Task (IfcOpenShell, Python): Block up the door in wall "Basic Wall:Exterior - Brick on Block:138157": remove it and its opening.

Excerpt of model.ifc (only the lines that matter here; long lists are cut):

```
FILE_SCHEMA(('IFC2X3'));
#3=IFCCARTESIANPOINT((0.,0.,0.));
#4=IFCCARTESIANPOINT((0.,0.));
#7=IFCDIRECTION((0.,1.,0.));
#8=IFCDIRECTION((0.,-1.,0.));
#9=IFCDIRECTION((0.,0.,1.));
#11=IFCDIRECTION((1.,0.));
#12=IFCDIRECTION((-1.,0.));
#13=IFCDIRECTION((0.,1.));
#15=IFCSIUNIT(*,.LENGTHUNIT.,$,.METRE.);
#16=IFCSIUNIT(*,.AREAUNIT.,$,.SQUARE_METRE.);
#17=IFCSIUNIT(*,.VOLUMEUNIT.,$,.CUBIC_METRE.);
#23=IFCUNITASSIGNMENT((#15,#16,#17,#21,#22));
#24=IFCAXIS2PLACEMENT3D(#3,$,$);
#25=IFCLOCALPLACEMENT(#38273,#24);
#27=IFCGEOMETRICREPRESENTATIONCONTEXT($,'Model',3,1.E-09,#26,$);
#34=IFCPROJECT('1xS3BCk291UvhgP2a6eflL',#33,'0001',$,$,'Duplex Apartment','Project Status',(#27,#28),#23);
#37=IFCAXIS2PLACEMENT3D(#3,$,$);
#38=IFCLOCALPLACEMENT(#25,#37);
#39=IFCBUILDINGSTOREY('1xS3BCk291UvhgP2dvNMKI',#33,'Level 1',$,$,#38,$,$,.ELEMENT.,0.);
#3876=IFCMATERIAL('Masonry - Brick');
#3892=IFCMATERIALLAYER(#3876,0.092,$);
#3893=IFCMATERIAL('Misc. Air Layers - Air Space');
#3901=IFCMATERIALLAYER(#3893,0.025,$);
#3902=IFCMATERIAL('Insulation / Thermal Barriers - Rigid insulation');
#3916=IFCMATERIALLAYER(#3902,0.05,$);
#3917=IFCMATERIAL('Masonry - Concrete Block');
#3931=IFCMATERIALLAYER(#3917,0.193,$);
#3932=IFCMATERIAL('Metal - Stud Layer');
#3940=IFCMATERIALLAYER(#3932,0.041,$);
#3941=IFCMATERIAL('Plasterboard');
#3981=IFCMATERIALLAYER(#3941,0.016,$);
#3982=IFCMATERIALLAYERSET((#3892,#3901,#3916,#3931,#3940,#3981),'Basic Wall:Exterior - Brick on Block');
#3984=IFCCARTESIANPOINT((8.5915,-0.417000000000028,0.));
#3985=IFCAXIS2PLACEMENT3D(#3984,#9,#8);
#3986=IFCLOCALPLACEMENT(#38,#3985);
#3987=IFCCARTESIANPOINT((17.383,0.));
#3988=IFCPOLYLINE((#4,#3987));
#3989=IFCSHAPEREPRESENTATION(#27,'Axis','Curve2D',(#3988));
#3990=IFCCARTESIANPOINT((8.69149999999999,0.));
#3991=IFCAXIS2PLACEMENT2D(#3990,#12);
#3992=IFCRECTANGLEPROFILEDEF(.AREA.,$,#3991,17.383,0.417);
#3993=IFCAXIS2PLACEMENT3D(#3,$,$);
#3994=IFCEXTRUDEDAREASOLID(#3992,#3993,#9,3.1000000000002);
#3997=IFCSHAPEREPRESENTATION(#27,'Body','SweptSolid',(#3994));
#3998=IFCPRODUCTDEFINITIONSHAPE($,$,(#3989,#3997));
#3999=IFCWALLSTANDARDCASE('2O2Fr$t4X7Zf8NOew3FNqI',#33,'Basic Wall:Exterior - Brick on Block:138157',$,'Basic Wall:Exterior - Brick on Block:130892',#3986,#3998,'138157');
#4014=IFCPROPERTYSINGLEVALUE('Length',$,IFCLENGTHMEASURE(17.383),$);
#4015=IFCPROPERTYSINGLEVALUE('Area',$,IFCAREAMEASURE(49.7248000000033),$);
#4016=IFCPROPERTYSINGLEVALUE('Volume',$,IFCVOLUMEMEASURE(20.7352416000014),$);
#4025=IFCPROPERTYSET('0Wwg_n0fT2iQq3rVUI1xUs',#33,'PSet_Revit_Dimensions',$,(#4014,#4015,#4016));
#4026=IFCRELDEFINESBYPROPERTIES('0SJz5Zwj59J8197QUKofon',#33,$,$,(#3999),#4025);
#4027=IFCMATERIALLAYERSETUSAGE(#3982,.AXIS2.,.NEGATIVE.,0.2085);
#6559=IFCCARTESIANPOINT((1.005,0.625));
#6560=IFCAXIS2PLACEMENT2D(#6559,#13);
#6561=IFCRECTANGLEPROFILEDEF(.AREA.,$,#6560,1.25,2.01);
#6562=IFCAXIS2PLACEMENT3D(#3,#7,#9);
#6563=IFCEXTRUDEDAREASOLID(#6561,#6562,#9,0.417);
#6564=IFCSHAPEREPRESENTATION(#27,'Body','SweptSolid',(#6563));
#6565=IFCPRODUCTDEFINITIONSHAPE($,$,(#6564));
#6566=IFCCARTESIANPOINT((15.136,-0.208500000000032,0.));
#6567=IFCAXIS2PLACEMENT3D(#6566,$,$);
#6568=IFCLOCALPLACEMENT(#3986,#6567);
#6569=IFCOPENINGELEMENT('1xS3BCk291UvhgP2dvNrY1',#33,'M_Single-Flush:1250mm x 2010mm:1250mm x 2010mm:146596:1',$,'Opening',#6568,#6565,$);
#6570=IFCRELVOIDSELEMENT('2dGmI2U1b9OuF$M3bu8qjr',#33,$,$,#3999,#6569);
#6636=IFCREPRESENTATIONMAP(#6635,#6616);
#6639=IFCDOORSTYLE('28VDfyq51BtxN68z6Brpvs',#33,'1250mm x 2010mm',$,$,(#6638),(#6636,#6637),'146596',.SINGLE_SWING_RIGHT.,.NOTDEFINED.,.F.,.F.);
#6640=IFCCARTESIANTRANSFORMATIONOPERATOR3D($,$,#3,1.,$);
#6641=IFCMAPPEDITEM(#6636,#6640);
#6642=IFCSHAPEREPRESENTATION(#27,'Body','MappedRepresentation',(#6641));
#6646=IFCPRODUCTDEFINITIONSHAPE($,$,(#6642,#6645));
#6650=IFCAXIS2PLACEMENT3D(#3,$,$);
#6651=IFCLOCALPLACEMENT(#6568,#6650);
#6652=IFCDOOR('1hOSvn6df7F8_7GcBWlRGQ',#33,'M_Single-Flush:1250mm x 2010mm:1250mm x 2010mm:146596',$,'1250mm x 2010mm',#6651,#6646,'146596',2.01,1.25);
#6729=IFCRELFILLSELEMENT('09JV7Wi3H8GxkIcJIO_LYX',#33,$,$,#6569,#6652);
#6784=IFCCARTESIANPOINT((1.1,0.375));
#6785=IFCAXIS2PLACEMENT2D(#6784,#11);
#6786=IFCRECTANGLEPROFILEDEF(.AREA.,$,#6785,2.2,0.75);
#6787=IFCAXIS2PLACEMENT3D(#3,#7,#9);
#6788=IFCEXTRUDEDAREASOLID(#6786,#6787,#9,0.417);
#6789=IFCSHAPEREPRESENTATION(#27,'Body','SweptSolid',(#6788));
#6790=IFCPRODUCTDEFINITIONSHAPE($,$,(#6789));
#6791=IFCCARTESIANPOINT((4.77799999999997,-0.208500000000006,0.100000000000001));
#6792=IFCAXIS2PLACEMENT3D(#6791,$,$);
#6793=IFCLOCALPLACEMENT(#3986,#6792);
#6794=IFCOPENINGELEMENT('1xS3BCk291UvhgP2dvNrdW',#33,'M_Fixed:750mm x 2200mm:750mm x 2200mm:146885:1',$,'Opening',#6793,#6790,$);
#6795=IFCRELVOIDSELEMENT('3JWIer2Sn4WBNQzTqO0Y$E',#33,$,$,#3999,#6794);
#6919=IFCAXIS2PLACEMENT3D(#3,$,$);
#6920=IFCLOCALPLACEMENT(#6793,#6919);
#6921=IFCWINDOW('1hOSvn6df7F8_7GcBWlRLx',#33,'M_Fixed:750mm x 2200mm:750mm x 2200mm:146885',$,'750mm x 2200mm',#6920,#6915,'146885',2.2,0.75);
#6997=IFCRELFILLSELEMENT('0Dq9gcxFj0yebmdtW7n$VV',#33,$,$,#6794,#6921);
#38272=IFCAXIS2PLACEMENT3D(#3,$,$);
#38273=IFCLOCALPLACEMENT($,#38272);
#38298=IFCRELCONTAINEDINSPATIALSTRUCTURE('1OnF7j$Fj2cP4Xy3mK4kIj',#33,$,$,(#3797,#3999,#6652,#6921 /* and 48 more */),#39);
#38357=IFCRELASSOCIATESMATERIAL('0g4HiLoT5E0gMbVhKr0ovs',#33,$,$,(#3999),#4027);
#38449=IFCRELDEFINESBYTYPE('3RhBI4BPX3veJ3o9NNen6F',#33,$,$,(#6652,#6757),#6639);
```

```python
import ifcopenshell
import ifcopenshell.api.feature
import ifcopenshell.api.pset
import ifcopenshell.api.root
import ifcopenshell.geom
import ifcopenshell.util.element
import ifcopenshell.util.shape
import ifcopenshell.util.unit

model = ifcopenshell.open("model.ifc")
area_scale = ifcopenshell.util.unit.calculate_unit_scale(model, "AREAUNIT")
volume_scale = ifcopenshell.util.unit.calculate_unit_scale(model, "VOLUMEUNIT")
settings = ifcopenshell.geom.settings()


def volume(element):
    """Net volume in cubic metres, openings subtracted."""
    shape = ifcopenshell.geom.create_shape(settings, element)
    return ifcopenshell.util.shape.get_volume(shape.geometry)


door = model.by_id(6652)
opening = door.FillsVoids[0].RelatingOpeningElement
wall = opening.VoidsElements[0].RelatingBuildingElement
before = volume(wall)

ifcopenshell.api.root.remove_product(model, product=door)
ifcopenshell.api.feature.remove_feature(model, feature=opening)

after = volume(wall)
thickness = 0.417  # wall thickness in metres

# Update the wall's stored quantities.
pset = model.by_id(ifcopenshell.util.element.get_pset(wall, "PSet_Revit_Dimensions", should_inherit=False)["id"])
ifcopenshell.api.pset.edit_pset(model, pset=pset, properties={
    "Area": model.create_entity("IfcAreaMeasure", after / thickness / area_scale),
    "Volume": model.create_entity("IfcVolumeMeasure", after / volume_scale),
})

print(f"wall volume {before:.3f} -> {after:.3f} m3")

model.write("model_edited.ifc")
```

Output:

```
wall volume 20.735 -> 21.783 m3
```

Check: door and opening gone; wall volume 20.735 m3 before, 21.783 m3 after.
